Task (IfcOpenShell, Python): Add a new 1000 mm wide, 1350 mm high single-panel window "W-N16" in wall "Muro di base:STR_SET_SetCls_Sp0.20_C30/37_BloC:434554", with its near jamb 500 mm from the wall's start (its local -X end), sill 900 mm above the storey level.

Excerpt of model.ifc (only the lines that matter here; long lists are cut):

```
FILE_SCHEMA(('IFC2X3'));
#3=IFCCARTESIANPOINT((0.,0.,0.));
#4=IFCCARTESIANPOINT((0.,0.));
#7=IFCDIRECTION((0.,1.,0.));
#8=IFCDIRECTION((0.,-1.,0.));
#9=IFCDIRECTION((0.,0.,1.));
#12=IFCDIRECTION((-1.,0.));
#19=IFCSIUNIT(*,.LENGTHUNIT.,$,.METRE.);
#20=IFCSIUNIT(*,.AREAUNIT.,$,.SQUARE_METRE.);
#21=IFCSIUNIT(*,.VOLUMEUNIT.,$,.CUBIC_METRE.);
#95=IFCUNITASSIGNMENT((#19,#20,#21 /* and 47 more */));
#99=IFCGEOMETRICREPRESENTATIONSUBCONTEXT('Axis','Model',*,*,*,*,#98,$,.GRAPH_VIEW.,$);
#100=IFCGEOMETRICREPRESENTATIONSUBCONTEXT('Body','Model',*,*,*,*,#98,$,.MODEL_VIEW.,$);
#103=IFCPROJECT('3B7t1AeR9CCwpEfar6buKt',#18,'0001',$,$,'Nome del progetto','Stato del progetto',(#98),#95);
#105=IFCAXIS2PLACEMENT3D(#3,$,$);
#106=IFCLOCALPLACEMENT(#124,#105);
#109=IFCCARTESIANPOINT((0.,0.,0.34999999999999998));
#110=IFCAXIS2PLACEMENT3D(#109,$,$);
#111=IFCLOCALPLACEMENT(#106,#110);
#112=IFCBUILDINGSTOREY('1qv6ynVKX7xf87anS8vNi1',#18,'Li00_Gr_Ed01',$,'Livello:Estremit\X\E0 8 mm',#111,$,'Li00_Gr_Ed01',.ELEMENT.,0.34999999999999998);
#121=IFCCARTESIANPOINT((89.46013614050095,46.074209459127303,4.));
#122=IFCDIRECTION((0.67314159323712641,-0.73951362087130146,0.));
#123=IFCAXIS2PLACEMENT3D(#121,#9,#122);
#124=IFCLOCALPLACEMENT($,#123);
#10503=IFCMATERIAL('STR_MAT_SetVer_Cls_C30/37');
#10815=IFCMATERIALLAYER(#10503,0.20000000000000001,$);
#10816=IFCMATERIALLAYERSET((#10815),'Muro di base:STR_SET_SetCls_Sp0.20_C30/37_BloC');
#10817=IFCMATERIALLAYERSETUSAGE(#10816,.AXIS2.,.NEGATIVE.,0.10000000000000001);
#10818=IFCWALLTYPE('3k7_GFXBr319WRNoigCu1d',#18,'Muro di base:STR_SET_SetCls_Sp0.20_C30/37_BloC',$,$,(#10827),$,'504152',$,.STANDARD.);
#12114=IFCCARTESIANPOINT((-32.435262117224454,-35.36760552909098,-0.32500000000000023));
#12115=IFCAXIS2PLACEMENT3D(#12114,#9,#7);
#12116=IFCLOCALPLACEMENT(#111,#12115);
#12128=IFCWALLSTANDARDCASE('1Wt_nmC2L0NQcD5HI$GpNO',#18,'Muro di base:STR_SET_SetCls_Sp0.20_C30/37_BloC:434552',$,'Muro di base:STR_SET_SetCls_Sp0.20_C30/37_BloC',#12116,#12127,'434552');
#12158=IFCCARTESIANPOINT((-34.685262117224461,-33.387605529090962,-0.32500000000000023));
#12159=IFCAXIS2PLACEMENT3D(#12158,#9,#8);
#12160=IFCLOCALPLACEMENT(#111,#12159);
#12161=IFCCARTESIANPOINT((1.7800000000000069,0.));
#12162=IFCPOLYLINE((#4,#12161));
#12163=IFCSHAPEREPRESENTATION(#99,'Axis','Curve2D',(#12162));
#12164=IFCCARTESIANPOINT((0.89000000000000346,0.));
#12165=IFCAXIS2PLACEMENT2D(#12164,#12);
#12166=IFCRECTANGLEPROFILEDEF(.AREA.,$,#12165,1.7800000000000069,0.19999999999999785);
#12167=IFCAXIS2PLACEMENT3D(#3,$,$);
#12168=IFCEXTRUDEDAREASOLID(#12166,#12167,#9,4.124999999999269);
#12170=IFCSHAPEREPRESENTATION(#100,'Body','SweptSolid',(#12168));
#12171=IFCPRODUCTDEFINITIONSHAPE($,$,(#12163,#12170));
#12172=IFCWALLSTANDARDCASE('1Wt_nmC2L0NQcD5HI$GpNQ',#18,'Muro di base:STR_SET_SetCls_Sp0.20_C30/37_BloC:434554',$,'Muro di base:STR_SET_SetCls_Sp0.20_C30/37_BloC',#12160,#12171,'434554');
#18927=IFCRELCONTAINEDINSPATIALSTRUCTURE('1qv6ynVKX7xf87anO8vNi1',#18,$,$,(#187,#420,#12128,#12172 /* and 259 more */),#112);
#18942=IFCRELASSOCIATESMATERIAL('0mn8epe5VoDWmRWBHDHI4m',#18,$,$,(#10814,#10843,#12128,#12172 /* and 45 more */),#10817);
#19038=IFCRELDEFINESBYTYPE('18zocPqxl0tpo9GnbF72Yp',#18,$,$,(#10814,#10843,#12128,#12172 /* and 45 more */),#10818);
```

```python
import numpy as np
import ifcopenshell
import ifcopenshell.api.feature
import ifcopenshell.api.geometry
import ifcopenshell.api.root
import ifcopenshell.api.spatial
import ifcopenshell.api.type
import ifcopenshell.geom
import ifcopenshell.util.element
import ifcopenshell.util.placement
import ifcopenshell.util.representation
import ifcopenshell.util.shape
import ifcopenshell.util.unit

model = ifcopenshell.open("model.ifc")
unit_scale = ifcopenshell.util.unit.calculate_unit_scale(model)
settings = ifcopenshell.geom.settings()


def volume(element):
    """Net volume in cubic metres, openings subtracted."""
    shape = ifcopenshell.geom.create_shape(settings, element)
    return ifcopenshell.util.shape.get_volume(shape.geometry)


wall = model.by_guid("1Wt_nmC2L0NQcD5HI$GpNQ")
storey = ifcopenshell.util.element.get_container(wall, ifc_class="IfcBuildingStorey")
context = ifcopenshell.util.representation.get_context(model, "Model", "Body", "MODEL_VIEW")
before = volume(wall)

width, height, from_end, sill = 1, 1.35, 0.5, 0.9  # metres

# The wall runs along its own X axis, and the end named is its -X end.
wall_shape = ifcopenshell.geom.create_shape(settings, wall)
x, y, z = ifcopenshell.util.shape.get_vertices(wall_shape.geometry).T
start = x.min() + from_end
face, thickness = float(y.min()), float(y.max() - y.min())
wall_matrix = ifcopenshell.util.placement.get_local_placement(wall.ObjectPlacement)
level = ifcopenshell.util.placement.get_local_placement(storey.ObjectPlacement)[2, 3]


def in_wall(x, y):
    """Placement at x, y metres in the wall's axes, at sill height."""
    matrix = wall_matrix.copy()
    matrix[:, 3] = wall_matrix @ np.array([x / unit_scale, y / unit_scale, 0.0, 1.0])
    matrix[2, 3] = level + sill / unit_scale
    return matrix


# Opening: a box that overshoots both wall faces by 50 mm.
opening = ifcopenshell.api.root.create_entity(model, ifc_class="IfcOpeningElement")
box = ifcopenshell.api.geometry.add_wall_representation(
    model, context=context, length=width, height=height, thickness=thickness + 0.1
)
ifcopenshell.api.geometry.assign_representation(model, product=opening, representation=box)
ifcopenshell.api.geometry.edit_object_placement(model, product=opening, matrix=in_wall(start, face - 0.05), is_si=False)
ifcopenshell.api.feature.add_feature(model, feature=opening, element=wall)

window = ifcopenshell.api.root.create_entity(model, ifc_class="IfcWindow", name="W-N16")
window.OverallWidth, window.OverallHeight = width / unit_scale, height / unit_scale
body = ifcopenshell.api.geometry.add_window_representation(
    model,
    context=context,
    overall_width=window.OverallWidth,
    overall_height=window.OverallHeight,
    partition_type="SINGLE_PANEL",
)
ifcopenshell.api.geometry.assign_representation(model, product=window, representation=body)
ifcopenshell.api.spatial.assign_container(model, products=[window], relating_structure=storey)
fills = ifcopenshell.api.feature.add_filling(model, opening=opening, element=window)
fills.OwnerHistory = window.OwnerHistory  # required in IFC2X3

# IFC2X3 keeps the operation on the window style.
style = ifcopenshell.api.root.create_entity(model, ifc_class="IfcWindowStyle", name="W-N16")
style.OperationType, style.ConstructionType = "SINGLE_PANEL", "NOTDEFINED"
style.ParameterTakesPrecedence = style.Sizeable = False
ifcopenshell.api.type.assign_type(model, related_objects=[window], relating_type=style)

# Centre the window in the wall's thickness.
ifcopenshell.api.geometry.edit_object_placement(model, product=window, matrix=in_wall(start, face), is_si=False)
window_shape = ifcopenshell.geom.create_shape(settings, window)
depth = ifcopenshell.util.shape.get_vertices(window_shape.geometry)[:, 1]
offset = face + thickness / 2 - (depth.min() + depth.max()) / 2
ifcopenshell.api.geometry.edit_object_placement(model, product=window, matrix=in_wall(start, offset), is_si=False)

after = volume(wall)

print(f"wall volume {before:.3f} -> {after:.3f} m3")

model.write("model-out.ifc")
```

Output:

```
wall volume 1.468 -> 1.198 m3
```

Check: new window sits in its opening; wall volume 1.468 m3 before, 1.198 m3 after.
